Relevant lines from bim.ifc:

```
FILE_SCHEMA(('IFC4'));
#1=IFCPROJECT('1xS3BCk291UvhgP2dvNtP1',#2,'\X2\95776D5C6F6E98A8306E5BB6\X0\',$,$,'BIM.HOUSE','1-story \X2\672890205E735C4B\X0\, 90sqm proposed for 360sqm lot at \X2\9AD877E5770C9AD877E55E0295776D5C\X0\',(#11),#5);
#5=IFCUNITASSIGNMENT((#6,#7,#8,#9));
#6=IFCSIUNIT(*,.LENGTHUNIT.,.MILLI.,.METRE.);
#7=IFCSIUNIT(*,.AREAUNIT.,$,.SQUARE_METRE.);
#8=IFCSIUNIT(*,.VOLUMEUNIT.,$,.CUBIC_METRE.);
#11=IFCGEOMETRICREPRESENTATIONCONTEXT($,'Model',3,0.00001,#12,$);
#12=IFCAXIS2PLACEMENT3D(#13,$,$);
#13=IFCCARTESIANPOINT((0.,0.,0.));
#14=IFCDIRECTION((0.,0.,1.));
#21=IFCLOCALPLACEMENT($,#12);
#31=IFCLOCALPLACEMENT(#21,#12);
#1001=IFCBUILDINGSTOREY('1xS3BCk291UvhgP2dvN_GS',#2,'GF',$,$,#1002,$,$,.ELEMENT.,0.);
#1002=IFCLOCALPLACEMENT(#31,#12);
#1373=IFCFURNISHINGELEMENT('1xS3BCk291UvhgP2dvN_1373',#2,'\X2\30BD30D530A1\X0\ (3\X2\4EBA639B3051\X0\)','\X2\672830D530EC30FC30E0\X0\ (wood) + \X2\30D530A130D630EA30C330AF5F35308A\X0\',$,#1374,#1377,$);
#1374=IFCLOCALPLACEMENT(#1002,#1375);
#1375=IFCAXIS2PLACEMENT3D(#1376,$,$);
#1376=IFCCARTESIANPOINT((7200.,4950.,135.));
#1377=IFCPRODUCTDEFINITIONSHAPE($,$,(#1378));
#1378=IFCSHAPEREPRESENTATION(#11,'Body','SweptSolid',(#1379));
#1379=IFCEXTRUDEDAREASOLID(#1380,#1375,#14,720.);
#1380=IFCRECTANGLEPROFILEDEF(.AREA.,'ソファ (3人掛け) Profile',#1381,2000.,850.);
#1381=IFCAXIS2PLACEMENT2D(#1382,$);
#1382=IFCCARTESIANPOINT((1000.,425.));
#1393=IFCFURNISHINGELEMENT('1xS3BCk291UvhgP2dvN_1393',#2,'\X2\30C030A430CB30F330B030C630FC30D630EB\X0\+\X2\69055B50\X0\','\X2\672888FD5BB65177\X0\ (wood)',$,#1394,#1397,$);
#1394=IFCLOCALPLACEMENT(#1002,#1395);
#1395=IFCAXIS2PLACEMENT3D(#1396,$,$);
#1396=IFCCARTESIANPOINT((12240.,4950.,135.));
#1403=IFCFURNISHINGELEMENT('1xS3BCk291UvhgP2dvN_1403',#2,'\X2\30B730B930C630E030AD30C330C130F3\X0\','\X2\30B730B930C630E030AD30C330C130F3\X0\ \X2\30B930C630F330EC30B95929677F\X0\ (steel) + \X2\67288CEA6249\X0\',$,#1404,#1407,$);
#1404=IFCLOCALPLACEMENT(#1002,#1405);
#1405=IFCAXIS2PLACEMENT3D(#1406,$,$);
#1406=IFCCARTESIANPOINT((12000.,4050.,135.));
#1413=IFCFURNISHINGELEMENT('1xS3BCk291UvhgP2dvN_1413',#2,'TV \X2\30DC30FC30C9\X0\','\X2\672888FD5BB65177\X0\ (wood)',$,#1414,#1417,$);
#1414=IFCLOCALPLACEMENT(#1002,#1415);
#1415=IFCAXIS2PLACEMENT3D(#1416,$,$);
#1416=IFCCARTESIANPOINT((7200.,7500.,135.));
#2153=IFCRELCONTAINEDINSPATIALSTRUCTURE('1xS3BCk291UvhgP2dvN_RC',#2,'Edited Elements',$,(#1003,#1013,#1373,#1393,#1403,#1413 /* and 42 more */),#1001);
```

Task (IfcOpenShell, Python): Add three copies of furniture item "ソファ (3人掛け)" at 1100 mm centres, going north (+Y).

```python
import numpy as np
import ifcopenshell
import ifcopenshell.api.geometry
import ifcopenshell.api.root
import ifcopenshell.util.element
import ifcopenshell.util.placement
import ifcopenshell.util.unit

model = ifcopenshell.open("bim.ifc")
unit_scale = ifcopenshell.util.unit.calculate_unit_scale(model)


def reuse_history(source, copy):
    """copy_class also copies each property set's owner history, people and application; keep the originals."""
    for rel in copy.IsDefinedBy:
        if rel.is_a("IfcRelDefinesByProperties") and (history := rel.RelatingPropertyDefinition.OwnerHistory):
            rel.RelatingPropertyDefinition.OwnerHistory = source.OwnerHistory
            ifcopenshell.util.element.remove_deep2(model, history)


source = model.by_guid("1xS3BCk291UvhgP2dvN_1373")
base = ifcopenshell.util.placement.get_local_placement(source.ObjectPlacement)
step = np.array([0.0, 1.0, 0.0]) * 1.1 / unit_scale

for i in range(1, 4):
    copy = ifcopenshell.api.root.copy_class(model, product=source)
    copy.Representation = ifcopenshell.util.element.copy_deep(
        model, source.Representation, exclude=["IfcGeometricRepresentationContext", "IfcRepresentationMap"]
    )
    reuse_history(source, copy)
    matrix = base.copy()
    matrix[:3, 3] += i * step
    print("added at", matrix[:3, 3].round(3) + 0.0)
    ifcopenshell.api.geometry.edit_object_placement(model, product=copy, matrix=matrix, is_si=False)

model.write("bim_v2.ifc")
```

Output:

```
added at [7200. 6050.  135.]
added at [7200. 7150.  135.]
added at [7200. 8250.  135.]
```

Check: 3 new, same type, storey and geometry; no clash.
